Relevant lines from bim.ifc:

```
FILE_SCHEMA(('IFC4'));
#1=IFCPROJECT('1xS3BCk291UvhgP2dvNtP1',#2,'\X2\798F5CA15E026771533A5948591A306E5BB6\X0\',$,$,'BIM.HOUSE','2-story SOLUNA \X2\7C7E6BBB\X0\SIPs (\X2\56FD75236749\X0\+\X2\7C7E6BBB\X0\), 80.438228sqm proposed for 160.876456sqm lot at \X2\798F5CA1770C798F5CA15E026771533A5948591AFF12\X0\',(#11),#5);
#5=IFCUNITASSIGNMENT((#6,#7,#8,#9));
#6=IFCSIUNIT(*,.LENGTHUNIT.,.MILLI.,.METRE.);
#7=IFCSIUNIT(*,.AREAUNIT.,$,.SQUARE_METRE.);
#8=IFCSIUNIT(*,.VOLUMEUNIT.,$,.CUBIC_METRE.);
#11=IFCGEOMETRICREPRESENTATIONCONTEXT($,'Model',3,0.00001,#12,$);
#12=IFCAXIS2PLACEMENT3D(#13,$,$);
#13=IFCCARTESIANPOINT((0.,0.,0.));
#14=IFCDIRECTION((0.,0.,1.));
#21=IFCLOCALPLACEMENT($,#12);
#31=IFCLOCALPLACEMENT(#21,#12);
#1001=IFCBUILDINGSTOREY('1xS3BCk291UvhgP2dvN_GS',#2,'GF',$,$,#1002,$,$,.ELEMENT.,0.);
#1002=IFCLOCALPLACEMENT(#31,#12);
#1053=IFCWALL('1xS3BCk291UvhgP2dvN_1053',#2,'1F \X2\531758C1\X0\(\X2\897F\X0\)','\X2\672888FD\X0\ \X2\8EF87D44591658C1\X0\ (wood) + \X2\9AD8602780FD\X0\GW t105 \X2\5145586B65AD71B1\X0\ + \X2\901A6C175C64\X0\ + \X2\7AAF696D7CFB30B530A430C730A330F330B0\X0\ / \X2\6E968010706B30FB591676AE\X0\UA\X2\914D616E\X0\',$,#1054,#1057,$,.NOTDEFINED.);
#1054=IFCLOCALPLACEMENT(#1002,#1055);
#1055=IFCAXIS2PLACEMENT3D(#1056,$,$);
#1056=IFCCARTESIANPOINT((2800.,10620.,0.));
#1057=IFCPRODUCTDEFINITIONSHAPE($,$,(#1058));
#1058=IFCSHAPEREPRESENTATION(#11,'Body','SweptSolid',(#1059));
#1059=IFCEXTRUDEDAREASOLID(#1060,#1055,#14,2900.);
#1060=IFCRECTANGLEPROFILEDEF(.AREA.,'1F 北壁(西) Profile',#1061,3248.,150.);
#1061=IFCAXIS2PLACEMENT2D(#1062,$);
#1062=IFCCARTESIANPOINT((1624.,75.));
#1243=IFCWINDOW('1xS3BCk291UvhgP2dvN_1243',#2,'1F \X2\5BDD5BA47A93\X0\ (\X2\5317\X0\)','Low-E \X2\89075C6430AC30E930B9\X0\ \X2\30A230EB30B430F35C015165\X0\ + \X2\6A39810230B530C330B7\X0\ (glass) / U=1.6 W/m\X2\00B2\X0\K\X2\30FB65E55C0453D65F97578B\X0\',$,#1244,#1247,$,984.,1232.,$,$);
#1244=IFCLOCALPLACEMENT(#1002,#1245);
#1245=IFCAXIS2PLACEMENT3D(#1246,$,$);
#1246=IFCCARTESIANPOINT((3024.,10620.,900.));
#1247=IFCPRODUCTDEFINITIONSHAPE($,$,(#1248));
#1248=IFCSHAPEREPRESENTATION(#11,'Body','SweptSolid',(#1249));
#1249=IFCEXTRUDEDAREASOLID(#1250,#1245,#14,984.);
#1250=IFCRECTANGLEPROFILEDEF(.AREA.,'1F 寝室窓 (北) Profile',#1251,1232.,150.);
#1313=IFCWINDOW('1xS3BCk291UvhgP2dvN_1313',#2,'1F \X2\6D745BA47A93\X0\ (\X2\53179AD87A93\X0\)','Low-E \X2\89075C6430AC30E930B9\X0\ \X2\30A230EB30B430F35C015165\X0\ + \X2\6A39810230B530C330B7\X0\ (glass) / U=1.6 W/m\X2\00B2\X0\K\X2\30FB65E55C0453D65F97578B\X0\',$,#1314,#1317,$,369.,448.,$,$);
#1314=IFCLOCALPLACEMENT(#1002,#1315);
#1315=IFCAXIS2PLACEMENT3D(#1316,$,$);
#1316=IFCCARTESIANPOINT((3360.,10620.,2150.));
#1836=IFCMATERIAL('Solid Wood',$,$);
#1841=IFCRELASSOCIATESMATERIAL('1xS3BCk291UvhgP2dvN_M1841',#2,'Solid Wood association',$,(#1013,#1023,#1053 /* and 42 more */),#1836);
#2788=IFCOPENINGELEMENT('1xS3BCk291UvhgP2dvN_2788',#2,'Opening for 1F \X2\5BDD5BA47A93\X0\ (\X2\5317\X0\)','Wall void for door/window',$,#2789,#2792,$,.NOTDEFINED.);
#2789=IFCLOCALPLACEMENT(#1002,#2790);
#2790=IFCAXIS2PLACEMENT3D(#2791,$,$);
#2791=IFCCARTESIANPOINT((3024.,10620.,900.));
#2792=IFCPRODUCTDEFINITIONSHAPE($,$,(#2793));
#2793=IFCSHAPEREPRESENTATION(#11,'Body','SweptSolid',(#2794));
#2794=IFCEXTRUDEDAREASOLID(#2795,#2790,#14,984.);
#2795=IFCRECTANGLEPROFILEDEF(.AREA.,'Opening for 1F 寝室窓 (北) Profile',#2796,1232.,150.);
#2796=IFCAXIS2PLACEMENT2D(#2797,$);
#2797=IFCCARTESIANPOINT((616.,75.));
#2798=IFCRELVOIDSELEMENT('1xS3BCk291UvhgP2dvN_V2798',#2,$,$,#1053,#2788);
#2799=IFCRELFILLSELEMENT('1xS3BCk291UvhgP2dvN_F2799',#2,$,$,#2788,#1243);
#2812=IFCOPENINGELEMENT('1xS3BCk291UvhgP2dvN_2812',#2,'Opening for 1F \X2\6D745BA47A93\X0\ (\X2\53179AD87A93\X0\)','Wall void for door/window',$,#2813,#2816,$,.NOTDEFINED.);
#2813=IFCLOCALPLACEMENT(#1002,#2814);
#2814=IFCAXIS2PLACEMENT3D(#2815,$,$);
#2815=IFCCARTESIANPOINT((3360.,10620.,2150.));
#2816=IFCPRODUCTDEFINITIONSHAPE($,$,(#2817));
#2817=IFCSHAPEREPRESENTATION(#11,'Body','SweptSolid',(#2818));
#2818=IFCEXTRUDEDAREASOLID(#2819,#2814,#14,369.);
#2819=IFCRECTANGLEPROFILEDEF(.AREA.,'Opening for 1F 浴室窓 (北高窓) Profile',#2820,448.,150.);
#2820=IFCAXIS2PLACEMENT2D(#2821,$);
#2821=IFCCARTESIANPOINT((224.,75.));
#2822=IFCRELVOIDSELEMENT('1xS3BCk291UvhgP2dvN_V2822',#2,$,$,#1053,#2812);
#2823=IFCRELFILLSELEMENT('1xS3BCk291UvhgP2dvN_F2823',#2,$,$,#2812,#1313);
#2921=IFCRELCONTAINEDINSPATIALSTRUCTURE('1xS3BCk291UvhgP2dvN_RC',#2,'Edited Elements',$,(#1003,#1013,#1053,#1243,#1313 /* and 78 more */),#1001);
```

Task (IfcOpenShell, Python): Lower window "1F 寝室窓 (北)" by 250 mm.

```python
import numpy as np
import ifcopenshell
import ifcopenshell.api.geometry
import ifcopenshell.util.placement
import ifcopenshell.util.unit

model = ifcopenshell.open("bim.ifc")
unit_scale = ifcopenshell.util.unit.calculate_unit_scale(model)

window = model.by_guid("1xS3BCk291UvhgP2dvN_1243")
opening = window.FillsVoids[0].RelatingOpeningElement
dz = -0.25 / unit_scale

shift = np.array([0.0, 0.0, dz])
# The window is not placed relative to its opening, so move both.
for product in (opening, window):
    matrix = ifcopenshell.util.placement.get_local_placement(product.ObjectPlacement)
    matrix[:3, 3] += shift
    ifcopenshell.api.geometry.edit_object_placement(model, product=product, matrix=matrix, is_si=False)

print(f"moved by {dz * unit_scale:+.3f} m")

model.write("bim_rev.ifc")
```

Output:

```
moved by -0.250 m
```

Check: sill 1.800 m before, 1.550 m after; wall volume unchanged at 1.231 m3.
